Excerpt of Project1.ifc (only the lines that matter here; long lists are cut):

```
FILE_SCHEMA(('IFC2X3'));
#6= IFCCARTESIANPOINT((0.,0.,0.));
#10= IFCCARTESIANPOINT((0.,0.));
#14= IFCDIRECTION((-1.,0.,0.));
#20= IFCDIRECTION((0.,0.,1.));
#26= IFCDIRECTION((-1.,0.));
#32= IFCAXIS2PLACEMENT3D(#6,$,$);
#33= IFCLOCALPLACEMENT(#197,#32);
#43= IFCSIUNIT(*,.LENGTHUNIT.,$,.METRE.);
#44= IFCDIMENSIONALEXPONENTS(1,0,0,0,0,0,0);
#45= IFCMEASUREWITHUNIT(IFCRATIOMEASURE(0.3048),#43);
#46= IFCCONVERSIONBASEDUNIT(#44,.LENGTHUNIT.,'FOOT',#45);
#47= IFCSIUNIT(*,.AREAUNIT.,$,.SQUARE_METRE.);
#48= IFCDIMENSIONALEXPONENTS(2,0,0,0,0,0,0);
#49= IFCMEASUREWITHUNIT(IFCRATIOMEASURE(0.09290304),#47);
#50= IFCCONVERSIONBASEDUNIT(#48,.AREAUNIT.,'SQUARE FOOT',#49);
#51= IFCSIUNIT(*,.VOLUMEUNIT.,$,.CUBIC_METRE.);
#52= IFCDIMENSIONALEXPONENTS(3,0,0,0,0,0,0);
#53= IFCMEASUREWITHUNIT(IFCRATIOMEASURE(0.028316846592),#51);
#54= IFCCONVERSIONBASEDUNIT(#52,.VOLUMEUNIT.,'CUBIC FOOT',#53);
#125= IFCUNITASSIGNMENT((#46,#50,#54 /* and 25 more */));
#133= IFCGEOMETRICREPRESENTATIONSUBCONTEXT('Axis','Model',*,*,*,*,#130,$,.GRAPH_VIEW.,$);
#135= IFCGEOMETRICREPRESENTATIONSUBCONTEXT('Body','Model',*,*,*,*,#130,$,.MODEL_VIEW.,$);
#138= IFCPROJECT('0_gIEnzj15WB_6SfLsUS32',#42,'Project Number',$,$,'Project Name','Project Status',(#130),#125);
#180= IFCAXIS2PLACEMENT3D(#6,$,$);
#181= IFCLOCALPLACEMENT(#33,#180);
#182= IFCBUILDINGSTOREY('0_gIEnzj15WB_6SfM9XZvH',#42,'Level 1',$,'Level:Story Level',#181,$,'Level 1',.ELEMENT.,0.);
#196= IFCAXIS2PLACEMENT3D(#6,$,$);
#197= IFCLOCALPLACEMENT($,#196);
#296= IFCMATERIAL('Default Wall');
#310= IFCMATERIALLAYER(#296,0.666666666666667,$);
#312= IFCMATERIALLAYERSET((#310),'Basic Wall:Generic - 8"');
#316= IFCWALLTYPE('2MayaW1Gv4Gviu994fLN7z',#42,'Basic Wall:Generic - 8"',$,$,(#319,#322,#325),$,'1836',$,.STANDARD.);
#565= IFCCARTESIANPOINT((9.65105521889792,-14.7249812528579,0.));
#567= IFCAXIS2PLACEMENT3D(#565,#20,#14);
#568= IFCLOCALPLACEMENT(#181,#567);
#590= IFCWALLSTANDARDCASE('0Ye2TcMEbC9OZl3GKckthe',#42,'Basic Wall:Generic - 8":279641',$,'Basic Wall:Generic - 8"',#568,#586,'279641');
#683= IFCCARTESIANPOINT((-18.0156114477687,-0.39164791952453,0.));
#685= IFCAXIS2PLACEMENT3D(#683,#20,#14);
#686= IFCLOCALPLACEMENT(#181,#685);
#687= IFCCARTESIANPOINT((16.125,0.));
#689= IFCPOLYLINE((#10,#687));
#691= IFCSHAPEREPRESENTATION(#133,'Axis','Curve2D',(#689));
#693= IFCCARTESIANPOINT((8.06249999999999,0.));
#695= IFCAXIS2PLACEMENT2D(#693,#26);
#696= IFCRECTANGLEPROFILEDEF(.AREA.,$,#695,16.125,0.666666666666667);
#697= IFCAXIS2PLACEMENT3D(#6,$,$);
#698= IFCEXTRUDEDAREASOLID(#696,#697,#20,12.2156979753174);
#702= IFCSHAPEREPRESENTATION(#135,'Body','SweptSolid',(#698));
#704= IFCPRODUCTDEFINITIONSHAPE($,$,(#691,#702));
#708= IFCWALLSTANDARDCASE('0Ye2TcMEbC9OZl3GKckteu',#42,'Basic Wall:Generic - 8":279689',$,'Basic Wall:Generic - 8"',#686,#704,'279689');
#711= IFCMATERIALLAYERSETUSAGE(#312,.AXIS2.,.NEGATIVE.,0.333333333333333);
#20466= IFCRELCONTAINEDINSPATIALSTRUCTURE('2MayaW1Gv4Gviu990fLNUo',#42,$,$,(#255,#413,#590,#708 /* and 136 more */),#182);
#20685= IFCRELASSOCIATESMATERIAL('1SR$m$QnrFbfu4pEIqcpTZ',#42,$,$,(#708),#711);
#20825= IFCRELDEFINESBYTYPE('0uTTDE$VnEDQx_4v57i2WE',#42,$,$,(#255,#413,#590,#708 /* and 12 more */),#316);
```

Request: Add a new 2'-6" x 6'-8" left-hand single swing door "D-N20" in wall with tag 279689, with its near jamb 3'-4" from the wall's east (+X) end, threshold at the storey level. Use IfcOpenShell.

```python
import numpy as np
import ifcopenshell
import ifcopenshell.api.feature
import ifcopenshell.api.geometry
import ifcopenshell.api.root
import ifcopenshell.api.spatial
import ifcopenshell.api.type
import ifcopenshell.geom
import ifcopenshell.util.element
import ifcopenshell.util.placement
import ifcopenshell.util.representation
import ifcopenshell.util.shape
import ifcopenshell.util.unit

model = ifcopenshell.open("Project1.ifc")
unit_scale = ifcopenshell.util.unit.calculate_unit_scale(model)
settings = ifcopenshell.geom.settings()


def volume(element):
    """Net volume in cubic metres, openings subtracted."""
    shape = ifcopenshell.geom.create_shape(settings, element)
    return ifcopenshell.util.shape.get_volume(shape.geometry)


wall = model.by_id(708)
storey = ifcopenshell.util.element.get_container(wall, ifc_class="IfcBuildingStorey")
context = ifcopenshell.util.representation.get_context(model, "Model", "Body", "MODEL_VIEW")
before = volume(wall)

width, height, from_end, sill = 0.762, 2.032, 1.016, 0.0  # metres

# The wall runs along its own X axis, and the end named is its -X end.
wall_shape = ifcopenshell.geom.create_shape(settings, wall)
x, y, z = ifcopenshell.util.shape.get_vertices(wall_shape.geometry).T
start = x.min() + from_end
face, thickness = float(y.min()), float(y.max() - y.min())
wall_matrix = ifcopenshell.util.placement.get_local_placement(wall.ObjectPlacement)
level = ifcopenshell.util.placement.get_local_placement(storey.ObjectPlacement)[2, 3]


def in_wall(x, y):
    """Placement at x, y metres in the wall's axes, at sill height."""
    matrix = wall_matrix.copy()
    matrix[:, 3] = wall_matrix @ np.array([x / unit_scale, y / unit_scale, 0.0, 1.0])
    matrix[2, 3] = level + sill / unit_scale
    return matrix


# Opening: a box that overshoots both wall faces by 50 mm.
opening = ifcopenshell.api.root.create_entity(model, ifc_class="IfcOpeningElement")
box = ifcopenshell.api.geometry.add_wall_representation(
    model, context=context, length=width, height=height, thickness=thickness + 0.1
)
ifcopenshell.api.geometry.assign_representation(model, product=opening, representation=box)
ifcopenshell.api.geometry.edit_object_placement(model, product=opening, matrix=in_wall(start, face - 0.05), is_si=False)
ifcopenshell.api.feature.add_feature(model, feature=opening, element=wall)

door = ifcopenshell.api.root.create_entity(model, ifc_class="IfcDoor", name="D-N20")
door.OverallWidth, door.OverallHeight = width / unit_scale, height / unit_scale
body = ifcopenshell.api.geometry.add_door_representation(
    model,
    context=context,
    overall_width=door.OverallWidth,
    overall_height=door.OverallHeight,
    operation_type="SINGLE_SWING_LEFT",
    lining_properties={"LiningDepth": thickness / unit_scale, "ThresholdDepth": thickness / unit_scale},
)
ifcopenshell.api.geometry.assign_representation(model, product=door, representation=body)
ifcopenshell.api.spatial.assign_container(model, products=[door], relating_structure=storey)
fills = ifcopenshell.api.feature.add_filling(model, opening=opening, element=door)
fills.OwnerHistory = door.OwnerHistory  # required in IFC2X3

# IFC2X3 keeps the operation on the door style.
style = ifcopenshell.api.root.create_entity(model, ifc_class="IfcDoorStyle", name="D-N20")
style.OperationType, style.ConstructionType = "SINGLE_SWING_LEFT", "NOTDEFINED"
style.ParameterTakesPrecedence = style.Sizeable = False
ifcopenshell.api.type.assign_type(model, related_objects=[door], relating_type=style)

# The lining spans the wall, so the door starts at the wall face.
ifcopenshell.api.geometry.edit_object_placement(model, product=door, matrix=in_wall(start, face), is_si=False)

after = volume(wall)

print(f"wall volume {before:.3f} -> {after:.3f} m3")

model.write("Project1_rev.ifc")
```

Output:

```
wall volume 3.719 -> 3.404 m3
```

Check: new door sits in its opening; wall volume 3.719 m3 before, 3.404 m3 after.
